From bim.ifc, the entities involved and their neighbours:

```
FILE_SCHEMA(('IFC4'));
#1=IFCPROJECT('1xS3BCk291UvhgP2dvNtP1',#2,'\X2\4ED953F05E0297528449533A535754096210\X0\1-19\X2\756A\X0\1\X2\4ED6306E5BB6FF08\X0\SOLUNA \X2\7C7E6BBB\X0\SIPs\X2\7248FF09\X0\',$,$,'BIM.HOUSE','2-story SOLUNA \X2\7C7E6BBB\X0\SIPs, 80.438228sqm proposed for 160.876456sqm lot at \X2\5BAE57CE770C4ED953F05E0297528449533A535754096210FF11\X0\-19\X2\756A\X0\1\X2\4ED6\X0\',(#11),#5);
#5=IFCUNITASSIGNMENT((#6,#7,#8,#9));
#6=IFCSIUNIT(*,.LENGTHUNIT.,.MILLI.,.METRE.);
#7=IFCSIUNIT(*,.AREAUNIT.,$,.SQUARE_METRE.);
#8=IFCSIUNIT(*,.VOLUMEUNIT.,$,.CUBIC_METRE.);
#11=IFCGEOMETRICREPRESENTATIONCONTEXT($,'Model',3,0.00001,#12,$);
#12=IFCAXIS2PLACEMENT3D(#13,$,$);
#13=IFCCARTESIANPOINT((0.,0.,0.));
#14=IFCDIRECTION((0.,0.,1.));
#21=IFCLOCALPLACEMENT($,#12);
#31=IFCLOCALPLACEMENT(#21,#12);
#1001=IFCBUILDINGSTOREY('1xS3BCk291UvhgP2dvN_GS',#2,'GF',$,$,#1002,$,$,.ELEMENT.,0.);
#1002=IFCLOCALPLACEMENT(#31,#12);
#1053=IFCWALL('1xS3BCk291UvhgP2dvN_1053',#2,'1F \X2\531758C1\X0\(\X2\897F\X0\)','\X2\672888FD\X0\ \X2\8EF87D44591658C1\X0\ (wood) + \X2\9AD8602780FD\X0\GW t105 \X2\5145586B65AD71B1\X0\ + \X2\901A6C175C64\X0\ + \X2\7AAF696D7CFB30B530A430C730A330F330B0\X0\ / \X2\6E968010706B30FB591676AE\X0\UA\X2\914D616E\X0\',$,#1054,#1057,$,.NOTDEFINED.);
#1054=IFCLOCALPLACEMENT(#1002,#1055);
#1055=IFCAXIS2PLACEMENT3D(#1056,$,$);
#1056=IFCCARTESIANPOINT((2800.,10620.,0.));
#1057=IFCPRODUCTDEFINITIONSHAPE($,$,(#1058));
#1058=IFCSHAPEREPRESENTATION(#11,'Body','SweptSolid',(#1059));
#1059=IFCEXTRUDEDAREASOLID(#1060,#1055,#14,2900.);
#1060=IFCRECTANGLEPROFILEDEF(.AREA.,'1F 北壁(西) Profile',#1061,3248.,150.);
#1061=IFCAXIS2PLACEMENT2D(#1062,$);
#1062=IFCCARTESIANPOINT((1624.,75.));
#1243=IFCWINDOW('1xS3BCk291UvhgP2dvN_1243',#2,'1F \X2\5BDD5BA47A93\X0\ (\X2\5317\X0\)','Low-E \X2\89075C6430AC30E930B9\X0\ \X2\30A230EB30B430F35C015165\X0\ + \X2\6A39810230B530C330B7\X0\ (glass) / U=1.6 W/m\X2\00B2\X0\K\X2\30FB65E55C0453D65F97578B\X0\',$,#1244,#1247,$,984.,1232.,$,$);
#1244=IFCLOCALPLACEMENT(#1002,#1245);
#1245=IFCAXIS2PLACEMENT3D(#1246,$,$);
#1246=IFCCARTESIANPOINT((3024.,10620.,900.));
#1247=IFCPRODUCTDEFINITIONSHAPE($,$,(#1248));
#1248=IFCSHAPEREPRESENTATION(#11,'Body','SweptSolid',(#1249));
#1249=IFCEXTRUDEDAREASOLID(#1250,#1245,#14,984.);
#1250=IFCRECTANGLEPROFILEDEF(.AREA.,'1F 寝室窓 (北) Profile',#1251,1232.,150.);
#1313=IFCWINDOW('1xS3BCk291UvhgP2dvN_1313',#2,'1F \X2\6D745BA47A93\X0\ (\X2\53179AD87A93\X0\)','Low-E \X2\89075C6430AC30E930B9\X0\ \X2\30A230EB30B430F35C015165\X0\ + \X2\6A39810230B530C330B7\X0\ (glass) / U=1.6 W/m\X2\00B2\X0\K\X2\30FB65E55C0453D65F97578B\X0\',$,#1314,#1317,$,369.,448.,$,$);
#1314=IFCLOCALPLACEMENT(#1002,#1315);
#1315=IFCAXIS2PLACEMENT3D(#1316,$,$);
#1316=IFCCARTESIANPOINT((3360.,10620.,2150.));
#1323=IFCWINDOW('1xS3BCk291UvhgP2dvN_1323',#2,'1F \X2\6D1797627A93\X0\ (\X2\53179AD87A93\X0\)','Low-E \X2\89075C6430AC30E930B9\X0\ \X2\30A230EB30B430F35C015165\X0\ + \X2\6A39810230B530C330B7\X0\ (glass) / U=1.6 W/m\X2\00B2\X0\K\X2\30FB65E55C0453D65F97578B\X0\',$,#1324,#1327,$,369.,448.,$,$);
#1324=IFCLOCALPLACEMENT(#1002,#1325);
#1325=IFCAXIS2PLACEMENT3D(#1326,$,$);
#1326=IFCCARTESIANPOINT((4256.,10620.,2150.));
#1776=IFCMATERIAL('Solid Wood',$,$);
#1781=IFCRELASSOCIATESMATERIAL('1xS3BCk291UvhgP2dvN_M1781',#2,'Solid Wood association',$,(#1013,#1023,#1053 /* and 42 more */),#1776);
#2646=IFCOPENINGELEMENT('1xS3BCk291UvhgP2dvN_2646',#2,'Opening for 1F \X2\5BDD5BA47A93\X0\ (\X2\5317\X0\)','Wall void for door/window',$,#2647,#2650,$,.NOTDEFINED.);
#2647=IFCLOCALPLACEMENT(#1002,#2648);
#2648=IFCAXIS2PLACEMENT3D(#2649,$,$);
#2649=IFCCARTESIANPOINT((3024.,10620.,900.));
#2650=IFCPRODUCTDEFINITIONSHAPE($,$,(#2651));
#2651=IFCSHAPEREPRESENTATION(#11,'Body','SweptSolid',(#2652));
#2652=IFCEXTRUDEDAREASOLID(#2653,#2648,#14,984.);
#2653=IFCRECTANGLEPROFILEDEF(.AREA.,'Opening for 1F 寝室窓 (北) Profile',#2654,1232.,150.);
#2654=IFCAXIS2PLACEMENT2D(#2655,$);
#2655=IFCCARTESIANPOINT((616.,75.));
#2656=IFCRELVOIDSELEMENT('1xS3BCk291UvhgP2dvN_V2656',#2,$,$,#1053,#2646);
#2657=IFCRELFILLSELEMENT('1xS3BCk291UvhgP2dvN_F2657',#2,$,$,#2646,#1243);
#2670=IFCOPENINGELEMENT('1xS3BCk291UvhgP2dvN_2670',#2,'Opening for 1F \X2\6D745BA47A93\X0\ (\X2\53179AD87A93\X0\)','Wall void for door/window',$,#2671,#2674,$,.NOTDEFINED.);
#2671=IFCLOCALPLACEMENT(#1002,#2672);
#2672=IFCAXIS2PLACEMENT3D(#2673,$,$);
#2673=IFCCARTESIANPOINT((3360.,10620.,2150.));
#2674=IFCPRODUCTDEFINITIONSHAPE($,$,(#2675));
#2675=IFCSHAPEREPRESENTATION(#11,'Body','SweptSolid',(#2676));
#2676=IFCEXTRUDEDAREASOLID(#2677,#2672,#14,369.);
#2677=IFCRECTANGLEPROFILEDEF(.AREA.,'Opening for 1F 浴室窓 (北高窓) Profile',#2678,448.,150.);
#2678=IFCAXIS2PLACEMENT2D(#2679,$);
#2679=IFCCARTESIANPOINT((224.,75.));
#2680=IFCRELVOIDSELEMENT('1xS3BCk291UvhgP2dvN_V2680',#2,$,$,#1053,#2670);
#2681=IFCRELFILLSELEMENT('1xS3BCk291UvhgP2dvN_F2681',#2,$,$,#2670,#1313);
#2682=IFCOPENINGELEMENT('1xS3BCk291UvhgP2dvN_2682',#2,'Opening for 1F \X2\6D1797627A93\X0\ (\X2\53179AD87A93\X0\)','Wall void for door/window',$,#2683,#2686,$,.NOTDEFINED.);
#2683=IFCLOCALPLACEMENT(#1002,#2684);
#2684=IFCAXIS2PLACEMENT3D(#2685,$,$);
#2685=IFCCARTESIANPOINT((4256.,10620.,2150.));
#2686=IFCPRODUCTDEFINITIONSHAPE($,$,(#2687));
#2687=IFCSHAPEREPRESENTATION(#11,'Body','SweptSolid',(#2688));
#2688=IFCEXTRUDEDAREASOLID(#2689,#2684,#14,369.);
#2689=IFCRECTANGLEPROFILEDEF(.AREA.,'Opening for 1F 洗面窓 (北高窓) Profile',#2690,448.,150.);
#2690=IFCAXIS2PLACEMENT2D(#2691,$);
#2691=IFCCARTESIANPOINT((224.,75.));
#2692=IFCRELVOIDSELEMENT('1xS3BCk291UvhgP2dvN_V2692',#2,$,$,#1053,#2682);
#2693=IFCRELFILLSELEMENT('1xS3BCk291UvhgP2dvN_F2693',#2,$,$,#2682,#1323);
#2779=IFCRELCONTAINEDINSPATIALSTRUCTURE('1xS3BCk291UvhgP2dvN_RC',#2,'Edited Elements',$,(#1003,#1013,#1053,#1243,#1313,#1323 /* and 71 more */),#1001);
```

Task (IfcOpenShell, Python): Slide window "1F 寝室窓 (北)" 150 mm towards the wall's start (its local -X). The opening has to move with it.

```python
import ifcopenshell
import ifcopenshell.api.geometry
import ifcopenshell.util.placement

model = ifcopenshell.open("bim.ifc")

window = model.by_guid("1xS3BCk291UvhgP2dvN_1243")
opening = window.FillsVoids[0].RelatingOpeningElement
wall = opening.VoidsElements[0].RelatingBuildingElement

wall_matrix = ifcopenshell.util.placement.get_local_placement(wall.ObjectPlacement)
shift = wall_matrix[:3, 0] * -150.0
before = ifcopenshell.util.placement.get_local_placement(window.ObjectPlacement)[:3, 3].copy()

# The window is not placed relative to its opening, so move both.
for product in (opening, window):
    matrix = ifcopenshell.util.placement.get_local_placement(product.ObjectPlacement)
    matrix[:3, 3] += shift
    ifcopenshell.api.geometry.edit_object_placement(model, product=product, matrix=matrix, is_si=False)

after = ifcopenshell.util.placement.get_local_placement(window.ObjectPlacement)[:3, 3]
print("window moved by", (after - before).round(3) + 0.0)

model.write("bim-out.ifc")
```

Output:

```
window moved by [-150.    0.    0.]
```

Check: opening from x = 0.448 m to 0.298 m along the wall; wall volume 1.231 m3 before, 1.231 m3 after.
